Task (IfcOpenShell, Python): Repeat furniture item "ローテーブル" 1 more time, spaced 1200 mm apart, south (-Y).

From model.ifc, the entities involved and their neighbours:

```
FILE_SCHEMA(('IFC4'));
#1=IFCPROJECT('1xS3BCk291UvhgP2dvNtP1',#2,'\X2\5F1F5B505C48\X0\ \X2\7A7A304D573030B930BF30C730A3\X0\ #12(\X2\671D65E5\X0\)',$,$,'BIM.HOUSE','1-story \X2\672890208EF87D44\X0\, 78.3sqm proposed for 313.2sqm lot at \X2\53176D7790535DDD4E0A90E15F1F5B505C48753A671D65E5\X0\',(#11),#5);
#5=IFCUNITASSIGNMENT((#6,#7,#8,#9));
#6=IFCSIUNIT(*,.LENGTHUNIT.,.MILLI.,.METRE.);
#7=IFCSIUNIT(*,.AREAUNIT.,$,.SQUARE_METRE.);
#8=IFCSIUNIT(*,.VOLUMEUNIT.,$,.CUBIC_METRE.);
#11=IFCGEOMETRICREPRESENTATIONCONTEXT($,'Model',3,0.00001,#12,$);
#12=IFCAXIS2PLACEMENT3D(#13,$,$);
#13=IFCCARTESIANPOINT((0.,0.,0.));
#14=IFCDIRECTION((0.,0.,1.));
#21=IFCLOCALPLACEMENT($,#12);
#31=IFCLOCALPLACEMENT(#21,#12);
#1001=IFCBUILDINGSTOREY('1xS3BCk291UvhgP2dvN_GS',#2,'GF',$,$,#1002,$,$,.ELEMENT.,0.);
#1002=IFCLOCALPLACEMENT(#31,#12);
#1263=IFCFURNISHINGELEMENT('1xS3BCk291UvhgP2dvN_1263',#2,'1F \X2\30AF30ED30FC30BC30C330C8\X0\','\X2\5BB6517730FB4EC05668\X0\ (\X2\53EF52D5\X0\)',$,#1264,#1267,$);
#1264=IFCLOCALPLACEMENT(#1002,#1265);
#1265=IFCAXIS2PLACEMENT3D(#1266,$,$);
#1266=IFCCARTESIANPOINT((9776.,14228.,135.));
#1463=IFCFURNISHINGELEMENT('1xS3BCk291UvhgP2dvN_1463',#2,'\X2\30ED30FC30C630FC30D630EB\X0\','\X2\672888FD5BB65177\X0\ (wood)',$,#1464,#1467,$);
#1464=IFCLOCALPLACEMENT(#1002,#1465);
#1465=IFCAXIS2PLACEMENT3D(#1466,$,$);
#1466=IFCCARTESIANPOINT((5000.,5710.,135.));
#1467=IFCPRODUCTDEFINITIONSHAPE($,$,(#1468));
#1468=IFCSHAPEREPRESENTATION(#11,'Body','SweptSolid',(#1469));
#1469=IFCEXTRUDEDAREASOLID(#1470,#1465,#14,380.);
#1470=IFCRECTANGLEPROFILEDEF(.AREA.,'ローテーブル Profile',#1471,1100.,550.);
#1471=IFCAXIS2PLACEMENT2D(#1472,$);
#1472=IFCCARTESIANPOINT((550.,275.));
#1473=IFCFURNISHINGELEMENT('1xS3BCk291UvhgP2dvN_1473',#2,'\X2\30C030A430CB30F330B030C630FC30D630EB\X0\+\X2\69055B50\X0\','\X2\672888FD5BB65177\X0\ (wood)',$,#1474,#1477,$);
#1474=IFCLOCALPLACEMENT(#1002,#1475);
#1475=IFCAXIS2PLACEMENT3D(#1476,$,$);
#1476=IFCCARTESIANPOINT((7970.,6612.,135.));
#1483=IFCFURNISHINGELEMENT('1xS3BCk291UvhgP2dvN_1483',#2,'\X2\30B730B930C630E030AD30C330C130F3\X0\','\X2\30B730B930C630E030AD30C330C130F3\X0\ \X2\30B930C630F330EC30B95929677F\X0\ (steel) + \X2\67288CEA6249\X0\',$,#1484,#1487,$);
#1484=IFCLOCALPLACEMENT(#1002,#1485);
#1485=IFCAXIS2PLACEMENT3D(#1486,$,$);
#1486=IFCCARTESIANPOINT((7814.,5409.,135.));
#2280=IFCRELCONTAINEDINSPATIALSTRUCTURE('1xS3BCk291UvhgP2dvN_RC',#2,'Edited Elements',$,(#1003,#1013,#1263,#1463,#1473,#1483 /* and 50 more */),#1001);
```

```python
import numpy as np
import ifcopenshell
import ifcopenshell.api.geometry
import ifcopenshell.api.root
import ifcopenshell.util.element
import ifcopenshell.util.placement

model = ifcopenshell.open("model.ifc")


def reuse_history(source, copy):
    """copy_class also copies each property set's owner history, people and application; keep the originals."""
    for rel in copy.IsDefinedBy:
        if rel.is_a("IfcRelDefinesByProperties") and (history := rel.RelatingPropertyDefinition.OwnerHistory):
            rel.RelatingPropertyDefinition.OwnerHistory = source.OwnerHistory
            ifcopenshell.util.element.remove_deep2(model, history)


source = model.by_guid("1xS3BCk291UvhgP2dvN_1463")
base = ifcopenshell.util.placement.get_local_placement(source.ObjectPlacement)
step = np.array([0.0, -1.0, 0.0]) * 1200.0

for i in range(1, 2):
    copy = ifcopenshell.api.root.copy_class(model, product=source)
    copy.Representation = ifcopenshell.util.element.copy_deep(
        model, source.Representation, exclude=["IfcGeometricRepresentationContext", "IfcRepresentationMap"]
    )
    reuse_history(source, copy)
    matrix = base.copy()
    matrix[:3, 3] += i * step
    print("added at", matrix[:3, 3].round(3) + 0.0)
    ifcopenshell.api.geometry.edit_object_placement(model, product=copy, matrix=matrix, is_si=False)

model.write("model-out.ifc")
```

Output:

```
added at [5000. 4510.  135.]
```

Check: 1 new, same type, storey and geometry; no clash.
